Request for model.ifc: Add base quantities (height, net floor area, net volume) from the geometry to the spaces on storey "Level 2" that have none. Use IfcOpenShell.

First a look at what the model holds.

```python
import ifcopenshell
import ifcopenshell.util.element
import ifcopenshell.util.unit

model = ifcopenshell.open("model.ifc")
print(model.schema)
for unit_type in ("LENGTHUNIT", "AREAUNIT", "VOLUMEUNIT"):
    print(unit_type, ifcopenshell.util.unit.calculate_unit_scale(model, unit_type))
storey = next(s for s in model.by_type("IfcBuildingStorey") if s.Name == "Level 2")
spaces = [e for e in ifcopenshell.util.element.get_decomposition(storey) if e.is_a("IfcSpace")]
for e in sorted(spaces, key=lambda e: e.id()):
    print(e.id(), e.is_a(), e.Name, list(ifcopenshell.util.element.get_psets(e, qtos_only=True)), sep=" | ")
```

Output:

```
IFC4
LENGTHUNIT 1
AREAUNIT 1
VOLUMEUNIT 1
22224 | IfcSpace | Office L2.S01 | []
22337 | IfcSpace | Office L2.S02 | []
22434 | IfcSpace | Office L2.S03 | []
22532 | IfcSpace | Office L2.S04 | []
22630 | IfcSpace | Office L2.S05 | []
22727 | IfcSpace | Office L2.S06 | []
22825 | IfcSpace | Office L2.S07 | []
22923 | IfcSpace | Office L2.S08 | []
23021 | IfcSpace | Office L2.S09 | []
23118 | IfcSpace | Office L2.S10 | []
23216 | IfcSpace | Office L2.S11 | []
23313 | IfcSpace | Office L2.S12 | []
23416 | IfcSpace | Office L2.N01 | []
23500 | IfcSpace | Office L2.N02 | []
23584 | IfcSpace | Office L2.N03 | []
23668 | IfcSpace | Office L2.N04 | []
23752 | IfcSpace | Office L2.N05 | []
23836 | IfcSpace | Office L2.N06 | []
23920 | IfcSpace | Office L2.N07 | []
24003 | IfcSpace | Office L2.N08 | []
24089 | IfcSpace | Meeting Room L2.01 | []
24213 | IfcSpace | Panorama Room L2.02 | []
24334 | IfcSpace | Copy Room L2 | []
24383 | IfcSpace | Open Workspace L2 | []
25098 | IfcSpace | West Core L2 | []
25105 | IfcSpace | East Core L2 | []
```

```python
import ifcopenshell
import ifcopenshell.api.pset
import ifcopenshell.geom
import ifcopenshell.util.element
import ifcopenshell.util.shape
import ifcopenshell.util.unit

model = ifcopenshell.open("model.ifc")
unit_scale = ifcopenshell.util.unit.calculate_unit_scale(model)
area_scale = ifcopenshell.util.unit.calculate_unit_scale(model, "AREAUNIT")
volume_scale = ifcopenshell.util.unit.calculate_unit_scale(model, "VOLUMEUNIT")
settings = ifcopenshell.geom.settings()

storey = next(s for s in model.by_type("IfcBuildingStorey") if s.Name == "Level 2")
spaces = [e for e in ifcopenshell.util.element.get_decomposition(storey) if e.is_a("IfcSpace")]

for e in sorted(spaces, key=lambda e: e.id()):
    if ifcopenshell.util.element.get_psets(e, qtos_only=True, should_inherit=False):
        continue
    # Geometry comes back in metres, in the element's own axes.
    shape = ifcopenshell.geom.create_shape(settings, e)
    values = {
        "Height": ifcopenshell.util.shape.get_z(shape.geometry) / unit_scale,
        "NetFloorArea": ifcopenshell.util.shape.get_footprint_area(shape.geometry) / area_scale,
        "NetVolume": ifcopenshell.util.shape.get_volume(shape.geometry) / volume_scale,
    }
    qto = ifcopenshell.api.pset.add_qto(model, product=e, name="Qto_SpaceBaseQuantities")
    ifcopenshell.api.pset.edit_qto(model, qto=qto, properties=values)
    print(e.id(), {k: round(v, 3) for k, v in values.items()})

model.write("model_updated.ifc")
```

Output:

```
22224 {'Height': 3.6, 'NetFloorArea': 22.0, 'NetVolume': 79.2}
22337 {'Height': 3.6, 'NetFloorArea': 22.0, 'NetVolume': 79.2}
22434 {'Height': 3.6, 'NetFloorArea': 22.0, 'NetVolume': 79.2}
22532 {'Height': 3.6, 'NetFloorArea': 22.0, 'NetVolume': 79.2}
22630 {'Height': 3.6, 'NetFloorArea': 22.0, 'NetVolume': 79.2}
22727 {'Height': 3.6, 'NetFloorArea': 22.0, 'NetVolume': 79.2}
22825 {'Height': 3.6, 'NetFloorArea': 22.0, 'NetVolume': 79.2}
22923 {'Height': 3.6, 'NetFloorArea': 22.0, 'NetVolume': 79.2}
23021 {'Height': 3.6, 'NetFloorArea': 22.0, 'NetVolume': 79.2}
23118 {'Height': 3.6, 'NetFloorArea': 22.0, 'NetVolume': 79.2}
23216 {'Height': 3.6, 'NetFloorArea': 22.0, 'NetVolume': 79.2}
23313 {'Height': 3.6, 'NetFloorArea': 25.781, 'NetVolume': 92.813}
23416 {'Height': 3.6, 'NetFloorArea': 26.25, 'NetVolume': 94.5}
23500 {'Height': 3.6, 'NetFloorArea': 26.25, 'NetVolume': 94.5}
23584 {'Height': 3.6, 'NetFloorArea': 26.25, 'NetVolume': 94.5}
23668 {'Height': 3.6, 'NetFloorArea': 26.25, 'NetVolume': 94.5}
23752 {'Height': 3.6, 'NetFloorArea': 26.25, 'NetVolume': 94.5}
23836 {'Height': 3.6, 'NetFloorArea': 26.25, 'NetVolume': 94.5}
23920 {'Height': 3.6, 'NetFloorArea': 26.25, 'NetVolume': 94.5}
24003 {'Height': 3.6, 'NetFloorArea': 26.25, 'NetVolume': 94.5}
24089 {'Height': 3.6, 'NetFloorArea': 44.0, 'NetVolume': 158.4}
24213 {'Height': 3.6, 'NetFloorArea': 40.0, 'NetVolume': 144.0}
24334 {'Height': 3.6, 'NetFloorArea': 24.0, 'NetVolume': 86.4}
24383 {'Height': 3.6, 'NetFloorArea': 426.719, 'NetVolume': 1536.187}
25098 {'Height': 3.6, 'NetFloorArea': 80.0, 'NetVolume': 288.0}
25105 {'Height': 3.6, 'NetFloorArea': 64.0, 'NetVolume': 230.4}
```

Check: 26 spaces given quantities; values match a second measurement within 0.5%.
